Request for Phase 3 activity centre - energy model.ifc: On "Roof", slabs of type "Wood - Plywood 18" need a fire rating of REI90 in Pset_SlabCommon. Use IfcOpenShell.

First a look at what the model holds.

```python
import ifcopenshell
import ifcopenshell.util.element

model = ifcopenshell.open("Phase 3 activity centre - energy model.ifc")
print(model.schema)
storey = next(s for s in model.by_type("IfcBuildingStorey") if s.Name == "Roof")
slabs = [e for e in ifcopenshell.util.element.get_decomposition(storey) if e.is_a("IfcSlab")]
seen = {}
for e in slabs:
    element_type = ifcopenshell.util.element.get_type(e)
    key = (element_type.Name if element_type != e and element_type else None, ifcopenshell.util.element.get_pset(e, "Pset_SlabCommon", "FireRating"))
    seen[key] = seen.get(key, 0) + 1
for (name, value), count in sorted(seen.items(), key=str):
    print(count, "x", name, "|", value)
```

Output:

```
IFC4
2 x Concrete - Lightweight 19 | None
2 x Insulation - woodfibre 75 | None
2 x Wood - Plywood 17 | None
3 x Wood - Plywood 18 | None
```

```python
import ifcopenshell
import ifcopenshell.api.pset
import ifcopenshell.util.element

model = ifcopenshell.open("Phase 3 activity centre - energy model.ifc")

storey = next(s for s in model.by_type("IfcBuildingStorey") if s.Name == "Roof")
slabs = [e for e in ifcopenshell.util.element.get_decomposition(storey) if e.is_a("IfcSlab")]

count = 0
for e in slabs:
    element_type = ifcopenshell.util.element.get_type(e)
    if element_type in (None, e) or element_type.Name != "Wood - Plywood 18":
        continue
    # add_pset returns the element's existing set when there is one.
    pset = ifcopenshell.api.pset.add_pset(model, product=e, name="Pset_SlabCommon")
    ifcopenshell.api.pset.edit_pset(model, pset=pset, properties={"FireRating": "REI90"})
    count += 1

print(count, "slabs updated")

model.write("Phase 3 activity centre - energy model-out.ifc")
```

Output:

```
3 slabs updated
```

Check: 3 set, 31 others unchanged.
